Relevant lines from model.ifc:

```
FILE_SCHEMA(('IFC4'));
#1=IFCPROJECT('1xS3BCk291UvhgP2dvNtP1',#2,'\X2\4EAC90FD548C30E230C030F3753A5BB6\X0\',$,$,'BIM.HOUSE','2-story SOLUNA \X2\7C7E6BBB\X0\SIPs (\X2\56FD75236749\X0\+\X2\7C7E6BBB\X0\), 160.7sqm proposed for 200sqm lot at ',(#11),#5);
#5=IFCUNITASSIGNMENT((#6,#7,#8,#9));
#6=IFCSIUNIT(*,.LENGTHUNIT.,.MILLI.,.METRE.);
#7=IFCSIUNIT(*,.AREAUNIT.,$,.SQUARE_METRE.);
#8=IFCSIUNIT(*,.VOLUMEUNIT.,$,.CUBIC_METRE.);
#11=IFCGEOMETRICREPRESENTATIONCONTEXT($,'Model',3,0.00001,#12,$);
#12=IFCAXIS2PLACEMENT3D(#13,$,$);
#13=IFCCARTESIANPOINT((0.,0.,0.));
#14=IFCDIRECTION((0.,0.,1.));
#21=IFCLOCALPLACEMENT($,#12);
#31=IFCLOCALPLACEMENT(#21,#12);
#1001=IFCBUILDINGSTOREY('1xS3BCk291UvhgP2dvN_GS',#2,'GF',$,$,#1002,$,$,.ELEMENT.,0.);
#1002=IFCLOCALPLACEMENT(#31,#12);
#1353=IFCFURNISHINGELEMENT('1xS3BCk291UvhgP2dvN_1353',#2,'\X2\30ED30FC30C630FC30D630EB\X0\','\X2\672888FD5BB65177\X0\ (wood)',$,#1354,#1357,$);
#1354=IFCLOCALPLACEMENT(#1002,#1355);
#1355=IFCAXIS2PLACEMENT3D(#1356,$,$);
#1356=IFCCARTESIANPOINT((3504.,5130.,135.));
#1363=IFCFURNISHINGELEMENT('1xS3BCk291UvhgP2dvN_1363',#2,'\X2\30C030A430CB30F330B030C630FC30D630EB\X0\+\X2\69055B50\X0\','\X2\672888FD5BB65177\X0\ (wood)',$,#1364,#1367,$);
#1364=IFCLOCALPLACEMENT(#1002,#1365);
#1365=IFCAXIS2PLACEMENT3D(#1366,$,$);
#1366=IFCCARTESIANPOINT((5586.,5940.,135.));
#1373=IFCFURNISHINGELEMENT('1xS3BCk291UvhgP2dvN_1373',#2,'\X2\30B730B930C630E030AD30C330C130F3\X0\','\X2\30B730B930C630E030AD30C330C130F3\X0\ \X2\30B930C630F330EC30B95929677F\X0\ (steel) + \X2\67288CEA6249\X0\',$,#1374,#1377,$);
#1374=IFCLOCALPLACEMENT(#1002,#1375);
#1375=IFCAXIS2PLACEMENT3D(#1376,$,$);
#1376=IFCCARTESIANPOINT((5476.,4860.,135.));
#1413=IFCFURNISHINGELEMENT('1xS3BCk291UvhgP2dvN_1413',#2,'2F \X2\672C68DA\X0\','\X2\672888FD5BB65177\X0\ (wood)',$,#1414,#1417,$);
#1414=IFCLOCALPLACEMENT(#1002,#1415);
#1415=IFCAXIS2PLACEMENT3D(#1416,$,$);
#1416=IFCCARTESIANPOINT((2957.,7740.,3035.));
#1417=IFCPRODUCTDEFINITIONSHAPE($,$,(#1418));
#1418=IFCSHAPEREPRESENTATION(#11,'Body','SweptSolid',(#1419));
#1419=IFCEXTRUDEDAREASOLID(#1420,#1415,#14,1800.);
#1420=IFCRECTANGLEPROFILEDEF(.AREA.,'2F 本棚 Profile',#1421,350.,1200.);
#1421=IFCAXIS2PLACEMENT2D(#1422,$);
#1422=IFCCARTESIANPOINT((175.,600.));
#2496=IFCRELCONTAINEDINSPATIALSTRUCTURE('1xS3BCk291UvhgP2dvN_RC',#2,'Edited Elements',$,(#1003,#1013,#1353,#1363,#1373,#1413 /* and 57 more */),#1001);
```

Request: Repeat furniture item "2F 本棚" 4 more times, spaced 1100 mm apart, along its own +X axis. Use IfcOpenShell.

```python
import ifcopenshell
import ifcopenshell.api.geometry
import ifcopenshell.api.root
import ifcopenshell.util.element
import ifcopenshell.util.placement
import ifcopenshell.util.unit

model = ifcopenshell.open("model.ifc")
unit_scale = ifcopenshell.util.unit.calculate_unit_scale(model)


def reuse_history(source, copy):
    """copy_class also copies each property set's owner history, people and application; keep the originals."""
    for rel in copy.IsDefinedBy:
        if rel.is_a("IfcRelDefinesByProperties") and (history := rel.RelatingPropertyDefinition.OwnerHistory):
            rel.RelatingPropertyDefinition.OwnerHistory = source.OwnerHistory
            ifcopenshell.util.element.remove_deep2(model, history)


source = model.by_guid("1xS3BCk291UvhgP2dvN_1413")
base = ifcopenshell.util.placement.get_local_placement(source.ObjectPlacement)
step = base[:3, 0] * 1.1 / unit_scale

for i in range(1, 5):
    copy = ifcopenshell.api.root.copy_class(model, product=source)
    copy.Representation = ifcopenshell.util.element.copy_deep(
        model, source.Representation, exclude=["IfcGeometricRepresentationContext", "IfcRepresentationMap"]
    )
    reuse_history(source, copy)
    matrix = base.copy()
    matrix[:3, 3] += i * step
    print("added at", matrix[:3, 3].round(3) + 0.0)
    ifcopenshell.api.geometry.edit_object_placement(model, product=copy, matrix=matrix, is_si=False)

model.write("model_updated.ifc")
```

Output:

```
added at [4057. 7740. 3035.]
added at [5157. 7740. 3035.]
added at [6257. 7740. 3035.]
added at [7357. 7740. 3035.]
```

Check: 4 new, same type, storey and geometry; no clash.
